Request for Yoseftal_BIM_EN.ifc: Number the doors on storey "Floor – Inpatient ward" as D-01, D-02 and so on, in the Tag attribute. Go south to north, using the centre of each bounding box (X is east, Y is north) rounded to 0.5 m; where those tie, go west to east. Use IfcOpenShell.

First a look at what the model holds.

```python
import ifcopenshell
import ifcopenshell.util.element
import ifcopenshell.util.placement

model = ifcopenshell.open("Yoseftal_BIM_EN.ifc")
print(model.schema)
storey = next(s for s in model.by_type("IfcBuildingStorey") if s.Name == "Floor – Inpatient ward")
doors = [e for e in ifcopenshell.util.element.get_decomposition(storey) if e.is_a("IfcDoor")]
for e in sorted(doors, key=lambda e: e.id()):
    origin = ifcopenshell.util.placement.get_local_placement(e.ObjectPlacement)[:3, 3]
    print(e.id(), e.Tag, e.Name, origin.round(2) + 0.0, sep=" | ")
```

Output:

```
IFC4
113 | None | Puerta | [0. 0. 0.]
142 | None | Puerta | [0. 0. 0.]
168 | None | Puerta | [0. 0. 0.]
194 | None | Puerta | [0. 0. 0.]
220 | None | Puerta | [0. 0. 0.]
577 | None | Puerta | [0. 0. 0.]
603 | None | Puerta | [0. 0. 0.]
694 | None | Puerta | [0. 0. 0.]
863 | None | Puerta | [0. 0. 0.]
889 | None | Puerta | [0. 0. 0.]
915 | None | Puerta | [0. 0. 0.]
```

```python
import ifcopenshell
import ifcopenshell.geom
import ifcopenshell.util.element
import ifcopenshell.util.shape

model = ifcopenshell.open("Yoseftal_BIM_EN.ifc")
settings = ifcopenshell.geom.settings()
settings.set("use-world-coords", True)


def centre(element):
    shape = ifcopenshell.geom.create_shape(settings, element)
    return ifcopenshell.util.shape.get_bbox_centroid(shape.geometry)


storey = next(s for s in model.by_type("IfcBuildingStorey") if s.Name == "Floor – Inpatient ward")
doors = [e for e in ifcopenshell.util.element.get_decomposition(storey) if e.is_a("IfcDoor")]

# Insertion points can sit at a corner or the storey origin, so sort by the geometry (in metres).
centres = {e: centre(e) for e in doors}
doors.sort(key=lambda e: (round(centres[e][1] / 0.5), centres[e][0]))

for i, e in enumerate(doors, start=1):
    number = f"D-{i:02d}"
    e.Tag = number
    print(e.id(), number)

model.write("Yoseftal_BIM_EN-out.ifc")
```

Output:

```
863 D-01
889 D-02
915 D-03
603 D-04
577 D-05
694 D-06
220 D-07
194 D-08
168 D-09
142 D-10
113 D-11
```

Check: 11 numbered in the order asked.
